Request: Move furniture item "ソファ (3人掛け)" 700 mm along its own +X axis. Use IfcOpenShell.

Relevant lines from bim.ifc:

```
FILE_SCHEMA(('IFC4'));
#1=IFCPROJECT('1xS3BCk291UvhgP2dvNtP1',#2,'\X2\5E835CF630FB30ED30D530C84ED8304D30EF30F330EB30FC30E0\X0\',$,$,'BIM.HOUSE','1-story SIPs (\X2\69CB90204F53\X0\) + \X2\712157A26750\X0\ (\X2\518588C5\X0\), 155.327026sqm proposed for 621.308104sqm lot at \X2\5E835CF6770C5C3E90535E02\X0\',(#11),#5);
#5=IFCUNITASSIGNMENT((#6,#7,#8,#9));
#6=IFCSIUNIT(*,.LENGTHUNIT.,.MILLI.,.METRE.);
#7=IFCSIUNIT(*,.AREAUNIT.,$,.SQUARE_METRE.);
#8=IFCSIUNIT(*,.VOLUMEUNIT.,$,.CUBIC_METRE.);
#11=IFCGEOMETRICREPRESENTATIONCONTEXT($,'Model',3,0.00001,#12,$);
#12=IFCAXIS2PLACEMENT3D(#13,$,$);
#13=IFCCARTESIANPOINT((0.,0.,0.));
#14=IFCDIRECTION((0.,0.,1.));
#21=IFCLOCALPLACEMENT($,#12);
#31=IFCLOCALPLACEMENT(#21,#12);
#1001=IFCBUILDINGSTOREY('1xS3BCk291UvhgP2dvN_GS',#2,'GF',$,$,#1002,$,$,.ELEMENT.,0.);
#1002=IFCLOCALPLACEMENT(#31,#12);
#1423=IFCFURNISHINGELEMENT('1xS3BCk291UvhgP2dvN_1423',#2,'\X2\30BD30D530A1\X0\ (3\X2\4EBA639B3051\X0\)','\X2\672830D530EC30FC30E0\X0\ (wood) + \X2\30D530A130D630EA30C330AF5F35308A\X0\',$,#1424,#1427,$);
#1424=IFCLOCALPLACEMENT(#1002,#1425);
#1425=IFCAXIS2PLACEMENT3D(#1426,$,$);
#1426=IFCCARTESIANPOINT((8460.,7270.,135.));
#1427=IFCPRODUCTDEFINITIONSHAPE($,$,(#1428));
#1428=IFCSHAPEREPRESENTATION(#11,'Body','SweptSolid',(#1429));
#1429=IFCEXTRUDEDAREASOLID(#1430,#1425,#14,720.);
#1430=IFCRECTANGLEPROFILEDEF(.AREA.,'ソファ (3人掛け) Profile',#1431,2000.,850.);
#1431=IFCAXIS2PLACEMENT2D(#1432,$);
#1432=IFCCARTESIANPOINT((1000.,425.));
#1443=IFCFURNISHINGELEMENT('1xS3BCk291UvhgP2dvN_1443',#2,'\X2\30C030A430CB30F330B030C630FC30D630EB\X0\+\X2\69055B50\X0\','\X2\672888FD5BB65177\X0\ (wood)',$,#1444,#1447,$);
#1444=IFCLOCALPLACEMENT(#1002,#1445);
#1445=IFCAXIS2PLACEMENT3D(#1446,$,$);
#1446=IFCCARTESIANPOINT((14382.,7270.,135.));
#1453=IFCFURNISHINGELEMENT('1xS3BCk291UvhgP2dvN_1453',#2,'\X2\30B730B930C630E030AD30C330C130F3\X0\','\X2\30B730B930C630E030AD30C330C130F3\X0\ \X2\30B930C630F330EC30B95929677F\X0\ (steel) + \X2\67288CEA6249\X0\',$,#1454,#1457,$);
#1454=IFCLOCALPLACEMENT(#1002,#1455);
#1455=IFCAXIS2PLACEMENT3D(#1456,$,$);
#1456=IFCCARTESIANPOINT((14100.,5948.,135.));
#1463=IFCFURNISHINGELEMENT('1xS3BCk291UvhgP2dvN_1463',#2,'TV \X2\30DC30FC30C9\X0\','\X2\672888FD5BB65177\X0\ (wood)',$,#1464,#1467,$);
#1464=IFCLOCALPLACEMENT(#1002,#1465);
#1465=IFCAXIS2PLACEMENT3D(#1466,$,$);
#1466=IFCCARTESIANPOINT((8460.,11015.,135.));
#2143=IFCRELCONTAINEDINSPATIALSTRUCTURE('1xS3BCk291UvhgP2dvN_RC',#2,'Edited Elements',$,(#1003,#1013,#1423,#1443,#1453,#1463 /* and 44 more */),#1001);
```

```python
import ifcopenshell
import ifcopenshell.api.geometry
import ifcopenshell.util.placement
import ifcopenshell.util.unit

model = ifcopenshell.open("bim.ifc")
unit_scale = ifcopenshell.util.unit.calculate_unit_scale(model)

item = model.by_guid("1xS3BCk291UvhgP2dvN_1423")
matrix = ifcopenshell.util.placement.get_local_placement(item.ObjectPlacement)
matrix[:3, 3] += matrix[:3, 0] * 0.7 / unit_scale
ifcopenshell.api.geometry.edit_object_placement(model, product=item, matrix=matrix, is_si=False)

print(ifcopenshell.util.placement.get_local_placement(item.ObjectPlacement).round(3) + 0.0)

model.write("bim-out.ifc")
```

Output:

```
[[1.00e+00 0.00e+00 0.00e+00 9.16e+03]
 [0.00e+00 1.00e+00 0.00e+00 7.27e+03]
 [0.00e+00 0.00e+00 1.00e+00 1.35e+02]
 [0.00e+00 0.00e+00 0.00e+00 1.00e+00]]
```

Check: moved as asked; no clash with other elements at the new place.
